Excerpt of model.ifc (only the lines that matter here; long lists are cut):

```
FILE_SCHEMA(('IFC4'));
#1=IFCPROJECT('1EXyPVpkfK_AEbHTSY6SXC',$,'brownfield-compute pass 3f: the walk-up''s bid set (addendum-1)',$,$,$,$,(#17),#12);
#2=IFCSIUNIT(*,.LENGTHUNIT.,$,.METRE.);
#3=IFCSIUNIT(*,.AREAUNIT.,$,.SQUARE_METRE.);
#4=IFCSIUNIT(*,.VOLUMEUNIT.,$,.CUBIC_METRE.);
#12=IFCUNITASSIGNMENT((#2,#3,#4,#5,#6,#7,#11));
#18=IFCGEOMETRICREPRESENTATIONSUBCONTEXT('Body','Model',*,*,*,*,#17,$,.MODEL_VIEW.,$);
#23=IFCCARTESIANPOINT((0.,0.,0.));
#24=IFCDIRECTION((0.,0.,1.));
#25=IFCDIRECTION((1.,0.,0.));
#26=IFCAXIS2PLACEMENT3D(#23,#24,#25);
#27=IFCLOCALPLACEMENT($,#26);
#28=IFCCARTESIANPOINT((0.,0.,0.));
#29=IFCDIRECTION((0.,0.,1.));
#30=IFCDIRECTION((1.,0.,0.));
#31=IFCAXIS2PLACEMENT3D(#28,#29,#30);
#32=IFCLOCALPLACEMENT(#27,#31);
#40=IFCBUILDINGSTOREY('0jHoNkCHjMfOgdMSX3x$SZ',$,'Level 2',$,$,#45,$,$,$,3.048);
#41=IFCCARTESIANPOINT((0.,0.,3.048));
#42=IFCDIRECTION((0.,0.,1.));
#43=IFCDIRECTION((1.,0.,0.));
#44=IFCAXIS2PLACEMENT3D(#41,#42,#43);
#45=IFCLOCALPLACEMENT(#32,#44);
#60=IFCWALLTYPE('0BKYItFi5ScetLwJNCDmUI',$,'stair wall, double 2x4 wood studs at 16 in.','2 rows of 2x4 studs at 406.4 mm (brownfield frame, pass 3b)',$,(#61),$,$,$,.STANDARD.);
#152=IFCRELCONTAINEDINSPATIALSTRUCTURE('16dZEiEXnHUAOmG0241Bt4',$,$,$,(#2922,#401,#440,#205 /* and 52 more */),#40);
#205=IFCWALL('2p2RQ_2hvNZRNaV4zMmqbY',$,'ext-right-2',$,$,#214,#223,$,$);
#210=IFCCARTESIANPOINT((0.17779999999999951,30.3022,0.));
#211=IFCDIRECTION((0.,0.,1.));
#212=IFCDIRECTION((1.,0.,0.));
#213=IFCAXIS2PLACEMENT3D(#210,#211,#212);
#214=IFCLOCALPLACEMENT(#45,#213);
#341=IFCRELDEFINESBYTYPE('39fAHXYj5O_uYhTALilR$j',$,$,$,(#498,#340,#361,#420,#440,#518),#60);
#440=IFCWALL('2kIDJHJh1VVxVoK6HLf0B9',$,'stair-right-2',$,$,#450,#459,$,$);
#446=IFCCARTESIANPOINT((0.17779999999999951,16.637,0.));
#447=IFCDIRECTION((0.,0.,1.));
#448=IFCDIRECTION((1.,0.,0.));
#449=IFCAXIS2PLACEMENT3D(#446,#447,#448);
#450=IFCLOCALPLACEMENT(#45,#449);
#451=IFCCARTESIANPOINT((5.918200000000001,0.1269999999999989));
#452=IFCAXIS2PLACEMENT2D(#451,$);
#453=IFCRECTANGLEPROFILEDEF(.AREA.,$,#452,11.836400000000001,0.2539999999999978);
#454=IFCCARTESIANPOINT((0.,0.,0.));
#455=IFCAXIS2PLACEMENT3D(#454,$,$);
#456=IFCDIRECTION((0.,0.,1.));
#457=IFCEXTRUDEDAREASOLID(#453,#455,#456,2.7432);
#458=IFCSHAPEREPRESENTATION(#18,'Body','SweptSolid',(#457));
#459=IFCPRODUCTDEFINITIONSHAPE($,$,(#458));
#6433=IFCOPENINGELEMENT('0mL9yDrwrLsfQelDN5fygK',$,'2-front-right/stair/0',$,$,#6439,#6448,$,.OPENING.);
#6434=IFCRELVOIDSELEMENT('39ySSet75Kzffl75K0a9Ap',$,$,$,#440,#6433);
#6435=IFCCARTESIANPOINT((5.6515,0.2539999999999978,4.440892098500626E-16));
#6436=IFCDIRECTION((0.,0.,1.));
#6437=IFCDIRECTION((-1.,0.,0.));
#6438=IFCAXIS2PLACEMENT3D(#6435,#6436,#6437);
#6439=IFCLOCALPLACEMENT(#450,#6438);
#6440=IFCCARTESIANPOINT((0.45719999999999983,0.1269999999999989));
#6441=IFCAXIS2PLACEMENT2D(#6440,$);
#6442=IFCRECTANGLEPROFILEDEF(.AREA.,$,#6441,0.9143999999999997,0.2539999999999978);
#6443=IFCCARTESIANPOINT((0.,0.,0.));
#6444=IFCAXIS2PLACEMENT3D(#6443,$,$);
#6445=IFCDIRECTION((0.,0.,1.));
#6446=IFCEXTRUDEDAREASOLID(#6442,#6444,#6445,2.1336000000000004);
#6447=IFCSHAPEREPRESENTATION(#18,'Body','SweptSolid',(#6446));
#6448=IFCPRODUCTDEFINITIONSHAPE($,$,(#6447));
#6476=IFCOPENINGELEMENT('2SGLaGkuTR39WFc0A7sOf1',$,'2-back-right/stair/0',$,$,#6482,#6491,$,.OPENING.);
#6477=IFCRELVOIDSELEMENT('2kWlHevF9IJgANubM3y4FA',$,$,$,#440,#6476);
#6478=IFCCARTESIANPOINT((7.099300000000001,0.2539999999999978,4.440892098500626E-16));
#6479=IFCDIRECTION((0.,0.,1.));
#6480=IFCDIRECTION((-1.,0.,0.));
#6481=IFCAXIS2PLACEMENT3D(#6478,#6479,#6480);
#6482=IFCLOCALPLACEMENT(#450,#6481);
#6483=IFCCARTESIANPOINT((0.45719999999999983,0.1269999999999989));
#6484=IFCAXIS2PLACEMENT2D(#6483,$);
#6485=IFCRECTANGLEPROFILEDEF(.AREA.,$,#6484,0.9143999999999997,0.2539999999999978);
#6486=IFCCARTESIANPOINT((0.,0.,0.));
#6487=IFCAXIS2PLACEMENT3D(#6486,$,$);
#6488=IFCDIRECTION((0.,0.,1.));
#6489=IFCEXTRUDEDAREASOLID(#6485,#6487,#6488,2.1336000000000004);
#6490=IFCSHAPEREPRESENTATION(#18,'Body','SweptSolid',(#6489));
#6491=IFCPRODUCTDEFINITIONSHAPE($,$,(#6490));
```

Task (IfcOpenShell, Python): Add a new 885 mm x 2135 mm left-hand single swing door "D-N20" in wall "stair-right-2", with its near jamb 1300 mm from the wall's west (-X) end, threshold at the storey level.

```python
import numpy as np
import ifcopenshell
import ifcopenshell.api.feature
import ifcopenshell.api.geometry
import ifcopenshell.api.root
import ifcopenshell.api.spatial
import ifcopenshell.geom
import ifcopenshell.util.element
import ifcopenshell.util.placement
import ifcopenshell.util.representation
import ifcopenshell.util.shape
import ifcopenshell.util.unit

model = ifcopenshell.open("model.ifc")
unit_scale = ifcopenshell.util.unit.calculate_unit_scale(model)
settings = ifcopenshell.geom.settings()


def volume(element):
    """Net volume in cubic metres, openings subtracted."""
    shape = ifcopenshell.geom.create_shape(settings, element)
    return ifcopenshell.util.shape.get_volume(shape.geometry)


wall = model.by_guid("2kIDJHJh1VVxVoK6HLf0B9")
storey = ifcopenshell.util.element.get_container(wall, ifc_class="IfcBuildingStorey")
context = ifcopenshell.util.representation.get_context(model, "Model", "Body", "MODEL_VIEW")
before = volume(wall)

width, height, from_end, sill = 0.885, 2.135, 1.3, 0.0  # metres

# The wall runs along its own X axis, and the end named is its -X end.
wall_shape = ifcopenshell.geom.create_shape(settings, wall)
x, y, z = ifcopenshell.util.shape.get_vertices(wall_shape.geometry).T
start = x.min() + from_end
face, thickness = float(y.min()), float(y.max() - y.min())
wall_matrix = ifcopenshell.util.placement.get_local_placement(wall.ObjectPlacement)
level = ifcopenshell.util.placement.get_local_placement(storey.ObjectPlacement)[2, 3]


def in_wall(x, y):
    """Placement at x, y metres in the wall's axes, at sill height."""
    matrix = wall_matrix.copy()
    matrix[:, 3] = wall_matrix @ np.array([x / unit_scale, y / unit_scale, 0.0, 1.0])
    matrix[2, 3] = level + sill / unit_scale
    return matrix


# Opening: a box that overshoots both wall faces by 50 mm.
opening = ifcopenshell.api.root.create_entity(model, ifc_class="IfcOpeningElement", predefined_type="OPENING")
box = ifcopenshell.api.geometry.add_wall_representation(
    model, context=context, length=width, height=height, thickness=thickness + 0.1
)
ifcopenshell.api.geometry.assign_representation(model, product=opening, representation=box)
ifcopenshell.api.geometry.edit_object_placement(model, product=opening, matrix=in_wall(start, face - 0.05), is_si=False)
ifcopenshell.api.feature.add_feature(model, feature=opening, element=wall)

door = ifcopenshell.api.root.create_entity(model, ifc_class="IfcDoor", name="D-N20", predefined_type="DOOR")
door.OverallWidth, door.OverallHeight = width / unit_scale, height / unit_scale
door.OperationType = "SINGLE_SWING_LEFT"
body = ifcopenshell.api.geometry.add_door_representation(
    model,
    context=context,
    overall_width=door.OverallWidth,
    overall_height=door.OverallHeight,
    operation_type="SINGLE_SWING_LEFT",
    lining_properties={"LiningDepth": thickness / unit_scale, "ThresholdDepth": thickness / unit_scale},
)
ifcopenshell.api.geometry.assign_representation(model, product=door, representation=body)
ifcopenshell.api.spatial.assign_container(model, products=[door], relating_structure=storey)
ifcopenshell.api.feature.add_filling(model, opening=opening, element=door)

# The lining spans the wall, so the door starts at the wall face.
ifcopenshell.api.geometry.edit_object_placement(model, product=door, matrix=in_wall(start, face), is_si=False)

after = volume(wall)

print(f"wall volume {before:.3f} -> {after:.3f} m3")

model.write("model_updated.ifc")
```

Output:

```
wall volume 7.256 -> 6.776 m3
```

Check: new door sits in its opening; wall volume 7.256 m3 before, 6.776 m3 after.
